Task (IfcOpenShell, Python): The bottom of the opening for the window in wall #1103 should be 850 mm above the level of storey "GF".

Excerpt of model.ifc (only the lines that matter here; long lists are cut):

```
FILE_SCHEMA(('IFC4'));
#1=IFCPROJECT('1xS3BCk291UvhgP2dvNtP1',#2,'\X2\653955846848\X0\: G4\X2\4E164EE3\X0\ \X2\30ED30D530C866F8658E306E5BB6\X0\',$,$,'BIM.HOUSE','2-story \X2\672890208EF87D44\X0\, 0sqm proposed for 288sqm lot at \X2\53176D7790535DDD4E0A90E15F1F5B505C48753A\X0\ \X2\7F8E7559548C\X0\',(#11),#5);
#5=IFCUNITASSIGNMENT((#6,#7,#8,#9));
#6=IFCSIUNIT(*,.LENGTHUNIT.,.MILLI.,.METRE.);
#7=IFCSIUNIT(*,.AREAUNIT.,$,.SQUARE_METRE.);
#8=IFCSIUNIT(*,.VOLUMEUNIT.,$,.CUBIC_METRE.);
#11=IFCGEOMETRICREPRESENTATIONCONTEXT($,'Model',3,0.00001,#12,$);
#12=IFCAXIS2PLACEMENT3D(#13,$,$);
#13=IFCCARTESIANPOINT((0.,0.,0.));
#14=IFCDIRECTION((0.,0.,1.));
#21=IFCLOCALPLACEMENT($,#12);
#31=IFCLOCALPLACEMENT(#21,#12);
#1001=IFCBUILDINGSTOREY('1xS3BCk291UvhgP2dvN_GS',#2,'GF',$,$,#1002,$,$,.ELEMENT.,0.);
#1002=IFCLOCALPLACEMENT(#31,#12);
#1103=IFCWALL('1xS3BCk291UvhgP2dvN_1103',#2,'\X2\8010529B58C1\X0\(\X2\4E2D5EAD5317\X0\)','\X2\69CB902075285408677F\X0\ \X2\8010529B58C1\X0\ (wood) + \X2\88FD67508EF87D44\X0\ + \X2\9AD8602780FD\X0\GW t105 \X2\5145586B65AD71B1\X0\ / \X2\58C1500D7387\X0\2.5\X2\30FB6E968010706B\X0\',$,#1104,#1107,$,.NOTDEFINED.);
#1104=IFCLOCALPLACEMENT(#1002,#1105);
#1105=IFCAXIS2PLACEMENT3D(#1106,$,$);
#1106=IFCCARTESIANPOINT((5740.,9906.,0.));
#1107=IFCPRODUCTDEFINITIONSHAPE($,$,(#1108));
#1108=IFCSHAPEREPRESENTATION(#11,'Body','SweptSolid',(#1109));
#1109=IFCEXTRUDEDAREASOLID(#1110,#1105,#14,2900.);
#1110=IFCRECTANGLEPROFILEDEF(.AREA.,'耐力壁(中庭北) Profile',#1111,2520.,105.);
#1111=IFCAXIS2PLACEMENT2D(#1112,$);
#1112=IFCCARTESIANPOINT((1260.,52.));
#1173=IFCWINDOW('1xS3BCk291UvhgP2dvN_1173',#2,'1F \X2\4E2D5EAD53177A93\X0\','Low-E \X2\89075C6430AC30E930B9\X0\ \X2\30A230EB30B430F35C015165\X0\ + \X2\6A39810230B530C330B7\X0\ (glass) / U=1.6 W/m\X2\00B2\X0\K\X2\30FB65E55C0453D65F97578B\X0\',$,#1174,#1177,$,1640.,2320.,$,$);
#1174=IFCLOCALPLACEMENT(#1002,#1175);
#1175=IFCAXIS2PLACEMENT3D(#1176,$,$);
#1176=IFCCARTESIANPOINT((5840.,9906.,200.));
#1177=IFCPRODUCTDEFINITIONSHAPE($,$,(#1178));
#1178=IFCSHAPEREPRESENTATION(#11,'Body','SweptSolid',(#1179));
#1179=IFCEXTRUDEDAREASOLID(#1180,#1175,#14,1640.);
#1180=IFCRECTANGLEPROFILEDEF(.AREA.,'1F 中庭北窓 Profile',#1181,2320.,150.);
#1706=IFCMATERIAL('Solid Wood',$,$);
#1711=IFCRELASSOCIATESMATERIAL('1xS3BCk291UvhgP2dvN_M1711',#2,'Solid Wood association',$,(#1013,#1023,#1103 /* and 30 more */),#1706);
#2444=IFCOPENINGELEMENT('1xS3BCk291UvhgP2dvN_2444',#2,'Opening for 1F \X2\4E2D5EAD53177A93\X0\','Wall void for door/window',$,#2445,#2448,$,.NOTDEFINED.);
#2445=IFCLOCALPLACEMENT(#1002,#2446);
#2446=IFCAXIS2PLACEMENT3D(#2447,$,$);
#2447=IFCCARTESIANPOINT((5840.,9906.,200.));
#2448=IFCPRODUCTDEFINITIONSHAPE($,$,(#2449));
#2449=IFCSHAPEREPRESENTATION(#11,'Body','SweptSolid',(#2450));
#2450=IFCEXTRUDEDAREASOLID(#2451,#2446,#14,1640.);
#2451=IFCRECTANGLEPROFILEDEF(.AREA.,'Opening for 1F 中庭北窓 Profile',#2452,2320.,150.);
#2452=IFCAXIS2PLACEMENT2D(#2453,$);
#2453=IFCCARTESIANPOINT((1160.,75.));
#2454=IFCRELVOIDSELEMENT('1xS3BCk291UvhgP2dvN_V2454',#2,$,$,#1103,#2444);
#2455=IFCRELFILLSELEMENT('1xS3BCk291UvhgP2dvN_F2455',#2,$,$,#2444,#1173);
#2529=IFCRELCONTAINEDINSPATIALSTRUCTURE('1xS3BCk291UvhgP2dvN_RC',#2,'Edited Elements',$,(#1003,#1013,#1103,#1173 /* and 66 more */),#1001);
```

```python
import numpy as np
import ifcopenshell
import ifcopenshell.api.geometry
import ifcopenshell.geom
import ifcopenshell.util.element
import ifcopenshell.util.placement
import ifcopenshell.util.shape
import ifcopenshell.util.unit

model = ifcopenshell.open("model.ifc")
unit_scale = ifcopenshell.util.unit.calculate_unit_scale(model)

window = model.by_id(1173)
opening = window.FillsVoids[0].RelatingOpeningElement
storey = ifcopenshell.util.element.get_container(window, ifc_class="IfcBuildingStorey")
level = ifcopenshell.util.placement.get_local_placement(storey.ObjectPlacement)[2, 3]

# The opening's origin need not be at the sill, so measure its lowest point.
shape = ifcopenshell.geom.create_shape(ifcopenshell.geom.settings(), opening)
bottom = ifcopenshell.util.shape.get_shape_bottom_elevation(shape, shape.geometry) / unit_scale
dz = level + 850.0 - bottom

shift = np.array([0.0, 0.0, dz])
# The window is not placed relative to its opening, so move both.
for product in (opening, window):
    matrix = ifcopenshell.util.placement.get_local_placement(product.ObjectPlacement)
    matrix[:3, 3] += shift
    ifcopenshell.api.geometry.edit_object_placement(model, product=product, matrix=matrix, is_si=False)

print(f"moved by {dz * unit_scale:+.3f} m")

model.write("model_updated.ifc")
```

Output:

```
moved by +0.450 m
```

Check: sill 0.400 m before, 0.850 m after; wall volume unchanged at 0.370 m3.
